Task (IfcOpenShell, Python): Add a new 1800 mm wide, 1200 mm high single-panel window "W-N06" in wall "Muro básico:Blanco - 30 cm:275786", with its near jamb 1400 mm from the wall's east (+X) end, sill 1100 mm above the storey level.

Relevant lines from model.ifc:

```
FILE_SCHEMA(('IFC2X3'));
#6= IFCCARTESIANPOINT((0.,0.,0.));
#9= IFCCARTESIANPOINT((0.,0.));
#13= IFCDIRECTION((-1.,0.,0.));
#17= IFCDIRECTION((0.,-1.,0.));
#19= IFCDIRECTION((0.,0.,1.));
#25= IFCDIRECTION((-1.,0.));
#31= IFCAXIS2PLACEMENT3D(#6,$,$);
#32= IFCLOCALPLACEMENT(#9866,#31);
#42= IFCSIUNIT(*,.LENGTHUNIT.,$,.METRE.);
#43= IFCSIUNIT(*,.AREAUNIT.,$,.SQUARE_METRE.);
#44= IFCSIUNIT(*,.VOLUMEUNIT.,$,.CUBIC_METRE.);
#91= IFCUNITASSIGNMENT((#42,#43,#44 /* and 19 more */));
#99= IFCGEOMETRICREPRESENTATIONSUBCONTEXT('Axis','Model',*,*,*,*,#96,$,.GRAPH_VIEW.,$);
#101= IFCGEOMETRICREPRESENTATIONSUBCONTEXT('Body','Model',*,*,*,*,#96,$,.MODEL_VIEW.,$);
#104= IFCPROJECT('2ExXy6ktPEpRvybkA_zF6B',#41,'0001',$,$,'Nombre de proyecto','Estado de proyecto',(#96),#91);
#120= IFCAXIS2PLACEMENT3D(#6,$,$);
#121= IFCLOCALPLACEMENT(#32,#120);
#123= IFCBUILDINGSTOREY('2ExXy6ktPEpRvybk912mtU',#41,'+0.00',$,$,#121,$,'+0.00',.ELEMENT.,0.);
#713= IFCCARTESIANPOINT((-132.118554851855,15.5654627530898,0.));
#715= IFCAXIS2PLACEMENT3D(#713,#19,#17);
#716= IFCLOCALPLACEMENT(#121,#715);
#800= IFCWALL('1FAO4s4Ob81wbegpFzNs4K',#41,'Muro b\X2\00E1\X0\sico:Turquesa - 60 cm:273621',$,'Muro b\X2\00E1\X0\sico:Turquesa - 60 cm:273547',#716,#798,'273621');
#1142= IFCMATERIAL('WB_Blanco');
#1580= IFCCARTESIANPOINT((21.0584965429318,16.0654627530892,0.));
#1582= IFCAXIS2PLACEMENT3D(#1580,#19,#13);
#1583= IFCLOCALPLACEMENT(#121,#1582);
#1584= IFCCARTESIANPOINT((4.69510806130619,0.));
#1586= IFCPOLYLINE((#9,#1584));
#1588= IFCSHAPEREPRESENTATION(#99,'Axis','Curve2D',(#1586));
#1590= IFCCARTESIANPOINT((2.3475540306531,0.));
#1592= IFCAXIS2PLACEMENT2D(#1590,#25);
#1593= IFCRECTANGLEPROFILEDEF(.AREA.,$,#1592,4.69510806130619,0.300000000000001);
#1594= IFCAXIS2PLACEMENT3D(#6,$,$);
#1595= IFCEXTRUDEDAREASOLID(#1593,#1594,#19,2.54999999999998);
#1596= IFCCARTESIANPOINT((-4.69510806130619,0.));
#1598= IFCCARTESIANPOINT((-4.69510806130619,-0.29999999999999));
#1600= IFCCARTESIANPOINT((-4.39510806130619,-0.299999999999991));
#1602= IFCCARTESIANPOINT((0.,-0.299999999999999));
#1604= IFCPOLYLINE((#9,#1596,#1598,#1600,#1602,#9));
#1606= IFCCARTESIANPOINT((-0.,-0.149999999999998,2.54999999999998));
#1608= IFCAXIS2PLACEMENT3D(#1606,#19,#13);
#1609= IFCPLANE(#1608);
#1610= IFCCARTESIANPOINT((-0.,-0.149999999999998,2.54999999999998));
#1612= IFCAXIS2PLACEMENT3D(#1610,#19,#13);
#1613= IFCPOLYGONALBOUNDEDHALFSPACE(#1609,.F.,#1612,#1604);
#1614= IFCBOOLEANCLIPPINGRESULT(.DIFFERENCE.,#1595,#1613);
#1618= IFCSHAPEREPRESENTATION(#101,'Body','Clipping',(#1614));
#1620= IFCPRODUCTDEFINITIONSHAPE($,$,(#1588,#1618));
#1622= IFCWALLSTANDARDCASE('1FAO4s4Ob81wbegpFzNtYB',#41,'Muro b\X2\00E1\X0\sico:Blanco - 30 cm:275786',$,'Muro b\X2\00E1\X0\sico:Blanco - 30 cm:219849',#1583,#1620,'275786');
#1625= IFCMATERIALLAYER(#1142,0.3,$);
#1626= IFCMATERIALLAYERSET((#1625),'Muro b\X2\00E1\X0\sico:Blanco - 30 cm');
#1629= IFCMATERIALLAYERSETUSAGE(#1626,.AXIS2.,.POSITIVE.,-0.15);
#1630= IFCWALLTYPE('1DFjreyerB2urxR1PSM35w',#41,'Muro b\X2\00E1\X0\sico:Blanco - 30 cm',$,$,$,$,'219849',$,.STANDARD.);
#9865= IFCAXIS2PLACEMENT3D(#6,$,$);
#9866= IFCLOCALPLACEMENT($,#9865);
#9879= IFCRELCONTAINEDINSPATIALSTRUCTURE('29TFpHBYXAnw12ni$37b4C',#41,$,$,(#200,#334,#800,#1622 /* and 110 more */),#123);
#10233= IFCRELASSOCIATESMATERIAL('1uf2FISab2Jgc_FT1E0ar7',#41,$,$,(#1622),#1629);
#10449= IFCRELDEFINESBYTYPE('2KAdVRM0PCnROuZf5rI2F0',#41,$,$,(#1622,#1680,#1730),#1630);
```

```python
import numpy as np
import ifcopenshell
import ifcopenshell.api.feature
import ifcopenshell.api.geometry
import ifcopenshell.api.root
import ifcopenshell.api.spatial
import ifcopenshell.api.type
import ifcopenshell.geom
import ifcopenshell.util.element
import ifcopenshell.util.placement
import ifcopenshell.util.representation
import ifcopenshell.util.shape
import ifcopenshell.util.unit

model = ifcopenshell.open("model.ifc")
unit_scale = ifcopenshell.util.unit.calculate_unit_scale(model)
settings = ifcopenshell.geom.settings()


def volume(element):
    """Net volume in cubic metres, openings subtracted."""
    shape = ifcopenshell.geom.create_shape(settings, element)
    return ifcopenshell.util.shape.get_volume(shape.geometry)


wall = model.by_guid("1FAO4s4Ob81wbegpFzNtYB")
storey = ifcopenshell.util.element.get_container(wall, ifc_class="IfcBuildingStorey")
context = ifcopenshell.util.representation.get_context(model, "Model", "Body", "MODEL_VIEW")
before = volume(wall)

width, height, from_end, sill = 1.8, 1.2, 1.4, 1.1  # metres

# The wall runs along its own X axis, and the end named is its -X end.
wall_shape = ifcopenshell.geom.create_shape(settings, wall)
x, y, z = ifcopenshell.util.shape.get_vertices(wall_shape.geometry).T
start = x.min() + from_end
face, thickness = float(y.min()), float(y.max() - y.min())
wall_matrix = ifcopenshell.util.placement.get_local_placement(wall.ObjectPlacement)
level = ifcopenshell.util.placement.get_local_placement(storey.ObjectPlacement)[2, 3]


def in_wall(x, y):
    """Placement at x, y metres in the wall's axes, at sill height."""
    matrix = wall_matrix.copy()
    matrix[:, 3] = wall_matrix @ np.array([x / unit_scale, y / unit_scale, 0.0, 1.0])
    matrix[2, 3] = level + sill / unit_scale
    return matrix


# Opening: a box that overshoots both wall faces by 50 mm.
opening = ifcopenshell.api.root.create_entity(model, ifc_class="IfcOpeningElement")
box = ifcopenshell.api.geometry.add_wall_representation(
    model, context=context, length=width, height=height, thickness=thickness + 0.1
)
ifcopenshell.api.geometry.assign_representation(model, product=opening, representation=box)
ifcopenshell.api.geometry.edit_object_placement(model, product=opening, matrix=in_wall(start, face - 0.05), is_si=False)
ifcopenshell.api.feature.add_feature(model, feature=opening, element=wall)

window = ifcopenshell.api.root.create_entity(model, ifc_class="IfcWindow", name="W-N06")
window.OverallWidth, window.OverallHeight = width / unit_scale, height / unit_scale
body = ifcopenshell.api.geometry.add_window_representation(
    model,
    context=context,
    overall_width=window.OverallWidth,
    overall_height=window.OverallHeight,
    partition_type="SINGLE_PANEL",
)
ifcopenshell.api.geometry.assign_representation(model, product=window, representation=body)
ifcopenshell.api.spatial.assign_container(model, products=[window], relating_structure=storey)
fills = ifcopenshell.api.feature.add_filling(model, opening=opening, element=window)
fills.OwnerHistory = window.OwnerHistory  # required in IFC2X3

# IFC2X3 keeps the operation on the window style.
style = ifcopenshell.api.root.create_entity(model, ifc_class="IfcWindowStyle", name="W-N06")
style.OperationType, style.ConstructionType = "SINGLE_PANEL", "NOTDEFINED"
style.ParameterTakesPrecedence = style.Sizeable = False
ifcopenshell.api.type.assign_type(model, related_objects=[window], relating_type=style)

# Centre the window in the wall's thickness.
ifcopenshell.api.geometry.edit_object_placement(model, product=window, matrix=in_wall(start, face), is_si=False)
window_shape = ifcopenshell.geom.create_shape(settings, window)
depth = ifcopenshell.util.shape.get_vertices(window_shape.geometry)[:, 1]
offset = face + thickness / 2 - (depth.min() + depth.max()) / 2
ifcopenshell.api.geometry.edit_object_placement(model, product=window, matrix=in_wall(start, offset), is_si=False)

after = volume(wall)

print(f"wall volume {before:.3f} -> {after:.3f} m3")

model.write("model_updated.ifc")
```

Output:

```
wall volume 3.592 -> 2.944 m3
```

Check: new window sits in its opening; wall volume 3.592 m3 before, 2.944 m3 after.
